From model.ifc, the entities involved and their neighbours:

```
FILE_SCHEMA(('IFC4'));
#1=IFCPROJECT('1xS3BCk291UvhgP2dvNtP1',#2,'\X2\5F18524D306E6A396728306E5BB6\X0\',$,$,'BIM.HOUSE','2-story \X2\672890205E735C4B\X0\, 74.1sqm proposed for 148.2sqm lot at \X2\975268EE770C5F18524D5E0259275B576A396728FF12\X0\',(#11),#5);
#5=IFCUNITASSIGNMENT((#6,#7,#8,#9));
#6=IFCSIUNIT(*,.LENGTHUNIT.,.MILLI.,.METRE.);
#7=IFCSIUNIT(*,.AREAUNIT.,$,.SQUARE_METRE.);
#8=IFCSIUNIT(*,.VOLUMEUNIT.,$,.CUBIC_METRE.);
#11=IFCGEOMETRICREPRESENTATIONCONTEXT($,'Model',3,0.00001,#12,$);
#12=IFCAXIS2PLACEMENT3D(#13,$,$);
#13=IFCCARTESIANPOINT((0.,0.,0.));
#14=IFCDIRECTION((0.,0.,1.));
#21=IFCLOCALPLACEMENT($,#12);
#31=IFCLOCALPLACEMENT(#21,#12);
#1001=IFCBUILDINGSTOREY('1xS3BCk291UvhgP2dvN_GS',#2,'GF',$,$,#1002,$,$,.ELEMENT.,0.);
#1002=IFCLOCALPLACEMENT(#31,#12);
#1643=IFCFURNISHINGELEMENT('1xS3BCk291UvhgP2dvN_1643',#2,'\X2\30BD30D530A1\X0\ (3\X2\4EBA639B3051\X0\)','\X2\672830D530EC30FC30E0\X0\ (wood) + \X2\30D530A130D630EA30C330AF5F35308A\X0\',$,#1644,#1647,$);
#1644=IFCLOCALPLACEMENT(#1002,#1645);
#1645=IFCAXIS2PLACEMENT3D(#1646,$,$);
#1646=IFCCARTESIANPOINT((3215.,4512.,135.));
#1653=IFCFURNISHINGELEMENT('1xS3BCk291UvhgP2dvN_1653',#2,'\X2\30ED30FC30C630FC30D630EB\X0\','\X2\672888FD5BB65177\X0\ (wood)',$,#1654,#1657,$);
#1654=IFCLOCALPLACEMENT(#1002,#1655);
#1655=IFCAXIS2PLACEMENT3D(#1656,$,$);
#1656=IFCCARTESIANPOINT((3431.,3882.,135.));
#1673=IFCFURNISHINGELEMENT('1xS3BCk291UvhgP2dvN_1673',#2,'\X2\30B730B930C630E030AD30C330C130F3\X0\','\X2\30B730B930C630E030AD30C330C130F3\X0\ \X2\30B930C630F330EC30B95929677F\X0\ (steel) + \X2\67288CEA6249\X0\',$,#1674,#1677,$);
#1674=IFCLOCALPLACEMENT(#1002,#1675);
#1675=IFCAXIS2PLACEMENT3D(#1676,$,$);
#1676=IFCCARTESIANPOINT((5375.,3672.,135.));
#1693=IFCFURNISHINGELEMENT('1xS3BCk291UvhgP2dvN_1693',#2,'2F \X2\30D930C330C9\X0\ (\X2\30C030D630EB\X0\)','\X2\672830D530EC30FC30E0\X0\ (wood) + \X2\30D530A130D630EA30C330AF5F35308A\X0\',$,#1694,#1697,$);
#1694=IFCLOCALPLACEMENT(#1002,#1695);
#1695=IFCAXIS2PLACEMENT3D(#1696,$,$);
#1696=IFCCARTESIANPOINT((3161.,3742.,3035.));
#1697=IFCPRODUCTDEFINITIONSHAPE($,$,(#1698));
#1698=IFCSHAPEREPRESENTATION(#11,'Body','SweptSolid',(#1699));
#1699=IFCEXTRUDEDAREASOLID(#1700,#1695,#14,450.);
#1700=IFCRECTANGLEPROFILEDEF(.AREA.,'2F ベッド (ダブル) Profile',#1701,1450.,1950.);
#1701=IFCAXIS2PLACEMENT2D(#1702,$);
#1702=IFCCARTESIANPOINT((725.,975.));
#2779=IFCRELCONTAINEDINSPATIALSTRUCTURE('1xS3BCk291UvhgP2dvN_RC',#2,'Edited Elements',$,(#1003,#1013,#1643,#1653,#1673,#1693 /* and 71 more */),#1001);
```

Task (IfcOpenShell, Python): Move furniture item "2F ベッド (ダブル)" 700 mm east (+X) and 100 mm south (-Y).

```python
import ifcopenshell
import ifcopenshell.api.geometry
import ifcopenshell.util.placement
import ifcopenshell.util.unit

model = ifcopenshell.open("model.ifc")
unit_scale = ifcopenshell.util.unit.calculate_unit_scale(model)

item = model.by_guid("1xS3BCk291UvhgP2dvN_1693")
matrix = ifcopenshell.util.placement.get_local_placement(item.ObjectPlacement)
matrix[0, 3] += 0.7 / unit_scale
matrix[1, 3] -= 0.1 / unit_scale
ifcopenshell.api.geometry.edit_object_placement(model, product=item, matrix=matrix, is_si=False)

print(ifcopenshell.util.placement.get_local_placement(item.ObjectPlacement).round(3) + 0.0)

model.write("model-out.ifc")
```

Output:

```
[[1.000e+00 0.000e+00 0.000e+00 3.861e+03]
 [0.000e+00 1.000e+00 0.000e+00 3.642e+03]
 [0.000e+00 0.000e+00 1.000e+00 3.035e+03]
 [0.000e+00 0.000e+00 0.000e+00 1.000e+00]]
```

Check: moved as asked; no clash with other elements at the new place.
